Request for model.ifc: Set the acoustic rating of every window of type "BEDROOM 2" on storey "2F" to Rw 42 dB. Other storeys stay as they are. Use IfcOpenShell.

First a look at what the model holds.

```python
import ifcopenshell
import ifcopenshell.util.element

model = ifcopenshell.open("model.ifc")
print(model.schema)
storey = next(s for s in model.by_type("IfcBuildingStorey") if s.Name == "2F")
windows = [e for e in ifcopenshell.util.element.get_decomposition(storey) if e.is_a("IfcWindow")]
seen = {}
for e in windows:
    element_type = ifcopenshell.util.element.get_type(e)
    key = (element_type.Name if element_type != e and element_type else None, ifcopenshell.util.element.get_pset(e, "Pset_WindowCommon", "AcousticRating"))
    seen[key] = seen.get(key, 0) + 1
for (name, value), count in sorted(seen.items(), key=str):
    print(count, "x", name, "|", value)
```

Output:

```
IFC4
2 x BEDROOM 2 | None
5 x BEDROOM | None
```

```python
import ifcopenshell
import ifcopenshell.api.pset
import ifcopenshell.util.element

model = ifcopenshell.open("model.ifc")

storey = next(s for s in model.by_type("IfcBuildingStorey") if s.Name == "2F")
windows = [e for e in ifcopenshell.util.element.get_decomposition(storey) if e.is_a("IfcWindow")]

count = 0
for e in windows:
    element_type = ifcopenshell.util.element.get_type(e)
    if element_type in (None, e) or element_type.Name != "BEDROOM 2":
        continue
    # add_pset returns the element's existing set when there is one.
    pset = ifcopenshell.api.pset.add_pset(model, product=e, name="Pset_WindowCommon")
    ifcopenshell.api.pset.edit_pset(model, pset=pset, properties={"AcousticRating": "Rw 42 dB"})
    count += 1

print(count, "windows updated")

model.write("model_rev.ifc")
```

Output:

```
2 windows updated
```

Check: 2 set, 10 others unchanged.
